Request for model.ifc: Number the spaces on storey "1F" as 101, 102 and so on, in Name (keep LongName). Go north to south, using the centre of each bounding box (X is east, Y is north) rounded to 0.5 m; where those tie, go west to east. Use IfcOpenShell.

First a look at what the model holds.

```python
import ifcopenshell
import ifcopenshell.util.element
import ifcopenshell.util.placement

model = ifcopenshell.open("model.ifc")
print(model.schema)
storey = next(s for s in model.by_type("IfcBuildingStorey") if s.Name == "1F")
spaces = [e for e in ifcopenshell.util.element.get_decomposition(storey) if e.is_a("IfcSpace")]
for e in sorted(spaces, key=lambda e: e.id()):
    origin = ifcopenshell.util.placement.get_local_placement(e.ObjectPlacement)[:3, 3]
    print(e.id(), e.Name, e.LongName, origin.round(2) + 0.0, sep=" | ")
```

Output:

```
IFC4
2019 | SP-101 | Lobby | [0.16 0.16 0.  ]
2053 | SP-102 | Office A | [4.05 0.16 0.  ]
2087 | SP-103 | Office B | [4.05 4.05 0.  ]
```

```python
import ifcopenshell
import ifcopenshell.geom
import ifcopenshell.util.element
import ifcopenshell.util.shape

model = ifcopenshell.open("model.ifc")
settings = ifcopenshell.geom.settings()
settings.set("use-world-coords", True)


def centre(element):
    shape = ifcopenshell.geom.create_shape(settings, element)
    return ifcopenshell.util.shape.get_bbox_centroid(shape.geometry)


storey = next(s for s in model.by_type("IfcBuildingStorey") if s.Name == "1F")
spaces = [e for e in ifcopenshell.util.element.get_decomposition(storey) if e.is_a("IfcSpace")]

# Insertion points can sit at a corner or the storey origin, so sort by the geometry (in metres).
centres = {e: centre(e) for e in spaces}
spaces.sort(key=lambda e: (-round(centres[e][1] / 0.5), centres[e][0]))

for i, e in enumerate(spaces, start=1):
    number = f"1{i:02d}"
    e.Name = number
    print(e.id(), number)

model.write("model_v2.ifc")
```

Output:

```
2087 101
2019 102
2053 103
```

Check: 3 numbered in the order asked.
